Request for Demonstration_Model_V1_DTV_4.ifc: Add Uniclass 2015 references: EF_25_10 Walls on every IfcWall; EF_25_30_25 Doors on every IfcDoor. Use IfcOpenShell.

First a look at what the model holds.

```python
import ifcopenshell

model = ifcopenshell.open("Demonstration_Model_V1_DTV_4.ifc")
print(model.schema)
print("classifications:", [c.Name for c in model.by_type("IfcClassification")])
for ifc_class in ("IfcDoor", "IfcRoof", "IfcStair", "IfcWall", "IfcWindow"):
    print(ifc_class, len(model.by_type(ifc_class)))
```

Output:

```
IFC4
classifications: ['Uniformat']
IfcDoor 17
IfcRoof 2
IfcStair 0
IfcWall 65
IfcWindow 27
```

```python
import ifcopenshell
import ifcopenshell.api.classification

model = ifcopenshell.open("Demonstration_Model_V1_DTV_4.ifc")

system = ifcopenshell.api.classification.add_classification(model, classification="Uniclass 2015")

codes = {
    "IfcWall": ("EF_25_10", "Walls"),
    "IfcDoor": ("EF_25_30_25", "Doors"),
}
for ifc_class, (code, name) in codes.items():
    products = model.by_type(ifc_class)
    ifcopenshell.api.classification.add_reference(
        model, products=products, classification=system, identification=code, name=name
    )
    print(code, len(products))

model.write("Demonstration_Model_V1_DTV_4_v2.ifc")
```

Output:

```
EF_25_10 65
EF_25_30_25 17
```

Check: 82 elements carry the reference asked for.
